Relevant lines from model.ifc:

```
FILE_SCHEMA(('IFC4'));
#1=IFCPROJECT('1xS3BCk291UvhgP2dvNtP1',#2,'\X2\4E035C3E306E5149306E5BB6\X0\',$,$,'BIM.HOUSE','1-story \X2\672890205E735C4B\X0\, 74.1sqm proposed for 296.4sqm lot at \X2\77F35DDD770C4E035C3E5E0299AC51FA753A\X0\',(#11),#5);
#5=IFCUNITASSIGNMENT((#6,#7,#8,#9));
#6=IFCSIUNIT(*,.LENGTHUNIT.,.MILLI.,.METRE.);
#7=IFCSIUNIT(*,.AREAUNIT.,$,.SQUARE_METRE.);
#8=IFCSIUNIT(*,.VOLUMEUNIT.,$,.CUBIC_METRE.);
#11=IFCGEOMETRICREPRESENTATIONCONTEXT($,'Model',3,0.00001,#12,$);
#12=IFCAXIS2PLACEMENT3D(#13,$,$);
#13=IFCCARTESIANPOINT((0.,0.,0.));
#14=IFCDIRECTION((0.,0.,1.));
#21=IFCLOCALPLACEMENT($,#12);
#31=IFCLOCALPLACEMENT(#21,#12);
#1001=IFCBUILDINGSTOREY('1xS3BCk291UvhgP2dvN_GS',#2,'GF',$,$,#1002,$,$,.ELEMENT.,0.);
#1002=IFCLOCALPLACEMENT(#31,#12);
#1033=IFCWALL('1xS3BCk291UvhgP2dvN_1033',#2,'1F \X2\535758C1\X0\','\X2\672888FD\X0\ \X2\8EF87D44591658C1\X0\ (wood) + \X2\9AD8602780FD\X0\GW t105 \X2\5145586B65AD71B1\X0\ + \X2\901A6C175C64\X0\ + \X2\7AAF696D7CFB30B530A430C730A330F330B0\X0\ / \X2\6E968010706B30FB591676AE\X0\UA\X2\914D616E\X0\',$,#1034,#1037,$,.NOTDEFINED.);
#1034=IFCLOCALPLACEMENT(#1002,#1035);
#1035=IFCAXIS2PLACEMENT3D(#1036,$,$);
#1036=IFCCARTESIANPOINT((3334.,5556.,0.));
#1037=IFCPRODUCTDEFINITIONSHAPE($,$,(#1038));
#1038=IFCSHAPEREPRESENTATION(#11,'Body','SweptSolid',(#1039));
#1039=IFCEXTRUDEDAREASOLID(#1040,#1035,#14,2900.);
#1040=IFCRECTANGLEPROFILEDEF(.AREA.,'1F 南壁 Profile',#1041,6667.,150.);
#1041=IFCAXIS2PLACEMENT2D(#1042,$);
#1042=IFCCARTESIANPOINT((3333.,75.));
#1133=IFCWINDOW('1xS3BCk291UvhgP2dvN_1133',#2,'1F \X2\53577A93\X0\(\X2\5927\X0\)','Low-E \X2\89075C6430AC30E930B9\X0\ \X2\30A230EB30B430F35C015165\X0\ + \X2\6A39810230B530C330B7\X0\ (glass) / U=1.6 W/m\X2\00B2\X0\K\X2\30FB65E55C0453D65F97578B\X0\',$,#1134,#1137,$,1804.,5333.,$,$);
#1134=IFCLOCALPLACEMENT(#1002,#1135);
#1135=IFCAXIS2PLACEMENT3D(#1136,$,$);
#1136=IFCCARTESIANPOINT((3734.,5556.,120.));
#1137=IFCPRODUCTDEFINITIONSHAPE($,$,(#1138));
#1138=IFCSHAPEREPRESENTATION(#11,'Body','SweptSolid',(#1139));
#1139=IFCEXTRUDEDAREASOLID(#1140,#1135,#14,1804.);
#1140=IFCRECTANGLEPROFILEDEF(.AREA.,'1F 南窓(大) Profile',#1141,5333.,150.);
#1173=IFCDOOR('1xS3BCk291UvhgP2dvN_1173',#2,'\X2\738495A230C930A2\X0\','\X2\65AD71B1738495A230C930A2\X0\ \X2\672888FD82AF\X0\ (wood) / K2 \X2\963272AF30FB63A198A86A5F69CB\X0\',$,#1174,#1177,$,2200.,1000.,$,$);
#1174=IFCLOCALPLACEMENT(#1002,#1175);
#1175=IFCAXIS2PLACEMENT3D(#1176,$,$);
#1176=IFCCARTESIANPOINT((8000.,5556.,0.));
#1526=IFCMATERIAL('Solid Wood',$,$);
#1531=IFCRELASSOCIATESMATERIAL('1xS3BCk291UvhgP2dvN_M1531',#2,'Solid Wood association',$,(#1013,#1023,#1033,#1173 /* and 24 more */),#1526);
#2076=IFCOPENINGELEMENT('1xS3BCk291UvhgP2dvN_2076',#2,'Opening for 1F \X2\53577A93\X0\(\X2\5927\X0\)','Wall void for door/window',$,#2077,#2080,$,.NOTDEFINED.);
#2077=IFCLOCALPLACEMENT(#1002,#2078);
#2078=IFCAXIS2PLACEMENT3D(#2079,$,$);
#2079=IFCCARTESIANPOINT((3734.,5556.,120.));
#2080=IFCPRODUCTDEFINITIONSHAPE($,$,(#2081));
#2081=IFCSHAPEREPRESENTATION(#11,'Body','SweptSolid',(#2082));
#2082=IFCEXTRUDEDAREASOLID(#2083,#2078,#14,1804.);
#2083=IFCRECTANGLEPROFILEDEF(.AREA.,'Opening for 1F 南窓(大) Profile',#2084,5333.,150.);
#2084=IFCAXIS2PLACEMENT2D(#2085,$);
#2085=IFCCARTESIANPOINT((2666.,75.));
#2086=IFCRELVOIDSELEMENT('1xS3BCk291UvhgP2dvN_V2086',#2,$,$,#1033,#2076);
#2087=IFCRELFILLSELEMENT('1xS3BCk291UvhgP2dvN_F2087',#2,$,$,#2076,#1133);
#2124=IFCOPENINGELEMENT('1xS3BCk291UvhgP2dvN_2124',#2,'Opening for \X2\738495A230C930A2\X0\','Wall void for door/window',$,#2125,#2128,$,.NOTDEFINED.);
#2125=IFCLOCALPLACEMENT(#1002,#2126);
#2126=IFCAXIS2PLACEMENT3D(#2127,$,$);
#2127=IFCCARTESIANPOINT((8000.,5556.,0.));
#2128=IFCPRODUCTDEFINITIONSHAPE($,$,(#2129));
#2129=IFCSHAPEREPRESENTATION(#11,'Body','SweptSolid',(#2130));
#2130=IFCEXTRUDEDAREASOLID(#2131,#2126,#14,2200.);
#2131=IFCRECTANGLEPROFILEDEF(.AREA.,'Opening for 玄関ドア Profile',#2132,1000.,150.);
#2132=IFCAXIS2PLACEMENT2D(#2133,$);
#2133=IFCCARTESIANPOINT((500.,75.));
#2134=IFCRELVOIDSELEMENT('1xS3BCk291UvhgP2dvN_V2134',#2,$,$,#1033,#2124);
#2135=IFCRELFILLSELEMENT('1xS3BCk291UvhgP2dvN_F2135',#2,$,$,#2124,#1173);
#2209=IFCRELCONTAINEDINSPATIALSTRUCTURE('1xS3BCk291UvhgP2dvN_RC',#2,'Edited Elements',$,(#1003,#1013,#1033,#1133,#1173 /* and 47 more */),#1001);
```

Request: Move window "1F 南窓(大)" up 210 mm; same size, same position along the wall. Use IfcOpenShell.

```python
import numpy as np
import ifcopenshell
import ifcopenshell.api.geometry
import ifcopenshell.util.placement
import ifcopenshell.util.unit

model = ifcopenshell.open("model.ifc")
unit_scale = ifcopenshell.util.unit.calculate_unit_scale(model)

window = model.by_id(1133)
opening = window.FillsVoids[0].RelatingOpeningElement
dz = 210.0

shift = np.array([0.0, 0.0, dz])
# The window is not placed relative to its opening, so move both.
for product in (opening, window):
    matrix = ifcopenshell.util.placement.get_local_placement(product.ObjectPlacement)
    matrix[:3, 3] += shift
    ifcopenshell.api.geometry.edit_object_placement(model, product=product, matrix=matrix, is_si=False)

print(f"moved by {dz * unit_scale:+.3f} m")

model.write("model_v2.ifc")
```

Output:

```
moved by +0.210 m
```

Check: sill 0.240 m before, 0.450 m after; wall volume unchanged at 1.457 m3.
